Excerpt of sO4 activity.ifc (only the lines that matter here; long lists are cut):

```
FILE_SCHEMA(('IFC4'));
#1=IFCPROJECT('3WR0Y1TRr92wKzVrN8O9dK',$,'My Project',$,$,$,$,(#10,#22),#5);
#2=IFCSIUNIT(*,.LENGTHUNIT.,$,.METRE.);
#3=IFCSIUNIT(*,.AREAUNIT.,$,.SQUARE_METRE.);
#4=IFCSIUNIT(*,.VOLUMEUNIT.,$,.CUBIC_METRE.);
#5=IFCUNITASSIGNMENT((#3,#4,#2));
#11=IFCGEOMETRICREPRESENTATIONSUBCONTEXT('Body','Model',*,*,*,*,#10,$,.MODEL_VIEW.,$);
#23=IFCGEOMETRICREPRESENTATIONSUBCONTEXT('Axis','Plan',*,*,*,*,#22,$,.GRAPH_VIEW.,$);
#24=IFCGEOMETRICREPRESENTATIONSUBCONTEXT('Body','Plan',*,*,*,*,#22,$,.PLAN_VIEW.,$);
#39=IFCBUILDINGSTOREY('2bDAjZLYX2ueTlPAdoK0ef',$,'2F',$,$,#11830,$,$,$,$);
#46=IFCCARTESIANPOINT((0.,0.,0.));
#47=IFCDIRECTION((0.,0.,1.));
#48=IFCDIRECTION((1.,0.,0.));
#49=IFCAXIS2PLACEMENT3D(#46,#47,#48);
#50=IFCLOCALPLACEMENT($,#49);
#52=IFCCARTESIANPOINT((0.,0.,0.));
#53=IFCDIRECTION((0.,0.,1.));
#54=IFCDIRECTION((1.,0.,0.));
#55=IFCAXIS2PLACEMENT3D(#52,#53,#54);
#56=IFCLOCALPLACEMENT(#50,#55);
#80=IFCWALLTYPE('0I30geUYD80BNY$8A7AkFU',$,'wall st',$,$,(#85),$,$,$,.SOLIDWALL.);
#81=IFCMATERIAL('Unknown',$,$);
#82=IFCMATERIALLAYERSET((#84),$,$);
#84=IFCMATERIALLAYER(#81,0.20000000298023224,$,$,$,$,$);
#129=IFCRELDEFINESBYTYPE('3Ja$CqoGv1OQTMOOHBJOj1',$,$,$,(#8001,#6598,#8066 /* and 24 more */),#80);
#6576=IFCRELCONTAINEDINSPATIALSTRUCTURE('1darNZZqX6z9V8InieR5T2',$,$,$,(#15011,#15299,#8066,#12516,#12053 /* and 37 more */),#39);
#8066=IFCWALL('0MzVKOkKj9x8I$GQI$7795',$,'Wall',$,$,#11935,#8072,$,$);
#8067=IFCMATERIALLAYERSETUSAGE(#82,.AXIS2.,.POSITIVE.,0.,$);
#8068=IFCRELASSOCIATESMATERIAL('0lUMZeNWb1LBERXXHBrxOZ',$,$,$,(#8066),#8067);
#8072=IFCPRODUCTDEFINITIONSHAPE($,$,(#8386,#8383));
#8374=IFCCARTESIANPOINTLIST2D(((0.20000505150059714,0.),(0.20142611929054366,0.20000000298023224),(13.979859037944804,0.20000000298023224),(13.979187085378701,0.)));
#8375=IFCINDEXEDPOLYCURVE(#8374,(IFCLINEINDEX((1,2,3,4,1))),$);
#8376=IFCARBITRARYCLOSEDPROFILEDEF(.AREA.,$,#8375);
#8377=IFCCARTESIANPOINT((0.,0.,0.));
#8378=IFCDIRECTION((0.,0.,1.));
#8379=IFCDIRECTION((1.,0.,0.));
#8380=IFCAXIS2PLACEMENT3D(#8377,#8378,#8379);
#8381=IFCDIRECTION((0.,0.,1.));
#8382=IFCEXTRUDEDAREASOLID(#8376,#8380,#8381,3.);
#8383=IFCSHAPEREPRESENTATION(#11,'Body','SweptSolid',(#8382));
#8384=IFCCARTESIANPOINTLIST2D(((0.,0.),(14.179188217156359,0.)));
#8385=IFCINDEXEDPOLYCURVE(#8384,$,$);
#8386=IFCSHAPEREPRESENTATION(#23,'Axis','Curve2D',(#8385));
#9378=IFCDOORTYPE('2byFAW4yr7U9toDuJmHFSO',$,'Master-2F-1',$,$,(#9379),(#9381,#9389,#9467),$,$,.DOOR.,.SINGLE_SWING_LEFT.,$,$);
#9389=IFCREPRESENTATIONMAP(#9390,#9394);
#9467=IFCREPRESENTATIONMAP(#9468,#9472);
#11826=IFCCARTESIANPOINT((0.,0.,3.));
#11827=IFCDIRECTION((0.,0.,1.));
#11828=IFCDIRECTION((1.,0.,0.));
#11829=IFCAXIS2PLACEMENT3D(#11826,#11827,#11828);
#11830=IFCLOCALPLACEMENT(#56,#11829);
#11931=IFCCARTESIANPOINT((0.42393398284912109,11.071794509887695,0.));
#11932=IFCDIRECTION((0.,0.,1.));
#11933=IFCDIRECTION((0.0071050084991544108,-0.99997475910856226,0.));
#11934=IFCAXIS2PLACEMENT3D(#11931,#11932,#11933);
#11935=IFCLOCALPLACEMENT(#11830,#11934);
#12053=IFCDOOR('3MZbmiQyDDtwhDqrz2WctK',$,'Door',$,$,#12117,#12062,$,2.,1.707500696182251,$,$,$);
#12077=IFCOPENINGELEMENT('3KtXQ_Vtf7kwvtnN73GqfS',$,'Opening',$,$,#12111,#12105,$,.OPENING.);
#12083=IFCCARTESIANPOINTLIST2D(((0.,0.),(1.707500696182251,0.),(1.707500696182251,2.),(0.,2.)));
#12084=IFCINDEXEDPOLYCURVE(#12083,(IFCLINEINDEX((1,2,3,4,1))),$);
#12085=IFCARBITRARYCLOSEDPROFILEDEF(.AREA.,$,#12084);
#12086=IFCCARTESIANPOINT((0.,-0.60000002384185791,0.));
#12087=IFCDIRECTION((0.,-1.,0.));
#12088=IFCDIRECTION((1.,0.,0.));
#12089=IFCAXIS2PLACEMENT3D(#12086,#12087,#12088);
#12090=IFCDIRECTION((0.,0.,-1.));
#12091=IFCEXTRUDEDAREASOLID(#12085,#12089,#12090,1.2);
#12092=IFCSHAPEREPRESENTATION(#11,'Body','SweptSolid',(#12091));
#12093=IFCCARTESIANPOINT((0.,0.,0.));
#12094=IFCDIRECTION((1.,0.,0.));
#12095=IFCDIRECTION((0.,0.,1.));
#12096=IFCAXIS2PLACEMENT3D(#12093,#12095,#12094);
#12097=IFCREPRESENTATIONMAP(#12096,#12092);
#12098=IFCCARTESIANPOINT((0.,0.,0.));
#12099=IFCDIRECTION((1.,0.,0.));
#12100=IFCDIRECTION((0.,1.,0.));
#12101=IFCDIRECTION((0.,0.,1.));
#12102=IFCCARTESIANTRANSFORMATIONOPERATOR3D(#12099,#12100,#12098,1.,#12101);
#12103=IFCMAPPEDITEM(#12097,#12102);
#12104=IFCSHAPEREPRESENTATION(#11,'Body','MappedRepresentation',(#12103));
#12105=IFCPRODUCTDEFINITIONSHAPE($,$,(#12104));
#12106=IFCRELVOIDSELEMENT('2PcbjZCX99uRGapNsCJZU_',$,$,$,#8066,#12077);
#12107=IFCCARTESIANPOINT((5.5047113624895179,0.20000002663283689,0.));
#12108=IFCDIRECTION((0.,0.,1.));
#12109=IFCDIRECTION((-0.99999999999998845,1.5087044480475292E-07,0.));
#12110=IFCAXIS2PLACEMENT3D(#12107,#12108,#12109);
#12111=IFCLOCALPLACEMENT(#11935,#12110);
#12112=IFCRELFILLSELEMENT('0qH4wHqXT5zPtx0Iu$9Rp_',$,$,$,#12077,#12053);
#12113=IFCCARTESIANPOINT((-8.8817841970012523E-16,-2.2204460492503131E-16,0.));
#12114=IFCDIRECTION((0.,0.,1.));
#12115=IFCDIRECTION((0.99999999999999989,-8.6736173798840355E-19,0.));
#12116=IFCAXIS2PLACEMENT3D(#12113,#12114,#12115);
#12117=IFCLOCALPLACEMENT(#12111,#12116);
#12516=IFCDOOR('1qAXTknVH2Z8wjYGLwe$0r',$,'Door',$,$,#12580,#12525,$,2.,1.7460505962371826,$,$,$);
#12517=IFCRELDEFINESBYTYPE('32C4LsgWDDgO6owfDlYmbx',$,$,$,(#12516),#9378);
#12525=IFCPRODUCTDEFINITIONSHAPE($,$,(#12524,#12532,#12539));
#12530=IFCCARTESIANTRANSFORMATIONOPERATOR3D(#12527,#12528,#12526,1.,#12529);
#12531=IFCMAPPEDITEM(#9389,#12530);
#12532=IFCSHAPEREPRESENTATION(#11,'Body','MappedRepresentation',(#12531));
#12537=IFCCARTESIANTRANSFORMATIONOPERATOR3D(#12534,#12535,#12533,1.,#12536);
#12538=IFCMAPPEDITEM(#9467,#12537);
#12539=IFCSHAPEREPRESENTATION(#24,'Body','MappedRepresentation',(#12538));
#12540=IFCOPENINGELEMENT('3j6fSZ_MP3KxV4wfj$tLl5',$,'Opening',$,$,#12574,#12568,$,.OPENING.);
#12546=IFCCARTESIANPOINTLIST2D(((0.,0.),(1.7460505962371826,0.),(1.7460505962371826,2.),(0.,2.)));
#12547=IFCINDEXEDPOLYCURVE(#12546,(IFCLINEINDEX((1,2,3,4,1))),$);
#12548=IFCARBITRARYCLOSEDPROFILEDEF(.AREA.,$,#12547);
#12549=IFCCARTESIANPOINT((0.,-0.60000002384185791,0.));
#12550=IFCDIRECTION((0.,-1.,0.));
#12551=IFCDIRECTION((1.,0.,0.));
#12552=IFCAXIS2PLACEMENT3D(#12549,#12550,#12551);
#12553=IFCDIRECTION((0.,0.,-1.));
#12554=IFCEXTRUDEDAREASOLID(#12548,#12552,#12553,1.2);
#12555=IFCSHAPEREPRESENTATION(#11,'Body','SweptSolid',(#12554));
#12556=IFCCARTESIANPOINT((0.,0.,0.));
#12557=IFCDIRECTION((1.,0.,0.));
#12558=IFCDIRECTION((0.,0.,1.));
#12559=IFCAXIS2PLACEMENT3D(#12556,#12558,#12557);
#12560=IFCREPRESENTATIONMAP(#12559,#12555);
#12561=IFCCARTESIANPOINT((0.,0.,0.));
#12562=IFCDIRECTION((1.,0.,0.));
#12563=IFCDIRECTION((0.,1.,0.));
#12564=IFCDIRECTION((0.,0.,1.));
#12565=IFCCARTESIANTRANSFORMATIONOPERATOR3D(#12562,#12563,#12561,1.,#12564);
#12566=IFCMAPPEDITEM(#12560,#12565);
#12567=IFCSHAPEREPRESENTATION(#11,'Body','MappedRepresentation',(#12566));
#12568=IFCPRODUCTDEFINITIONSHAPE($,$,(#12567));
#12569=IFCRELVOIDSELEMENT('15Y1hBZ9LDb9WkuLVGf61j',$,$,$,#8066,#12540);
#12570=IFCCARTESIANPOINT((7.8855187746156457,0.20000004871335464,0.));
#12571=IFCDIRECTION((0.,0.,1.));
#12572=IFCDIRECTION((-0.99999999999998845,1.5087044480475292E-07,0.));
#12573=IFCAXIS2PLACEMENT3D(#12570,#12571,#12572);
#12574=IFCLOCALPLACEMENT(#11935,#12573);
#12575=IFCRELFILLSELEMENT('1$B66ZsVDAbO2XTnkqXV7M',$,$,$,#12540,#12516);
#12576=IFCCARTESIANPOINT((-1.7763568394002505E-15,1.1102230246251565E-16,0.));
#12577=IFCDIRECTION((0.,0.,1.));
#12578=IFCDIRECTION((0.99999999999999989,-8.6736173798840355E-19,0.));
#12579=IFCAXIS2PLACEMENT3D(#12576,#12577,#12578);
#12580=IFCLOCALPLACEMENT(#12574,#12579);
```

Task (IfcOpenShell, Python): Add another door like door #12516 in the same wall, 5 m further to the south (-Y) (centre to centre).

```python
import ifcopenshell
import ifcopenshell.api.feature
import ifcopenshell.api.geometry
import ifcopenshell.api.root
import ifcopenshell.geom
import ifcopenshell.util.element
import ifcopenshell.util.placement
import ifcopenshell.util.shape
import ifcopenshell.util.unit

model = ifcopenshell.open("sO4 activity.ifc")
unit_scale = ifcopenshell.util.unit.calculate_unit_scale(model)
settings = ifcopenshell.geom.settings()


def volume(element):
    """Net volume in cubic metres, openings subtracted."""
    shape = ifcopenshell.geom.create_shape(settings, element)
    return ifcopenshell.util.shape.get_volume(shape.geometry)


door = model.by_guid("1qAXTknVH2Z8wjYGLwe$0r")
opening = door.FillsVoids[0].RelatingOpeningElement
wall = opening.VoidsElements[0].RelatingBuildingElement
before = volume(wall)
shift = ifcopenshell.util.placement.get_local_placement(wall.ObjectPlacement)[:3, 0] * 5 / unit_scale

# copy_class copies the void relationship, type, container and properties, but no geometry.
new_opening = ifcopenshell.api.root.copy_class(model, product=opening)
new_opening.Representation = ifcopenshell.util.element.copy_deep(
    model, opening.Representation, exclude=["IfcGeometricRepresentationContext", "IfcRepresentationMap"]
)
new_door = ifcopenshell.api.root.copy_class(model, product=door)
new_door.Representation = ifcopenshell.util.element.copy_deep(
    model, door.Representation, exclude=["IfcGeometricRepresentationContext", "IfcRepresentationMap"]
)
ifcopenshell.api.feature.add_filling(model, opening=new_opening, element=new_door)

for old, new in ((opening, new_opening), (door, new_door)):
    matrix = ifcopenshell.util.placement.get_local_placement(old.ObjectPlacement)
    matrix[:3, 3] += shift
    ifcopenshell.api.geometry.edit_object_placement(model, product=new, matrix=matrix, is_si=False)

after = volume(wall)

print(f"wall volume {before:.3f} -> {after:.3f} m3")

model.write("sO4 activity_updated.ifc")
```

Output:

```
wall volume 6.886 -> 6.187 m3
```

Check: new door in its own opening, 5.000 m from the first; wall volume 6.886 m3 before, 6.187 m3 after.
